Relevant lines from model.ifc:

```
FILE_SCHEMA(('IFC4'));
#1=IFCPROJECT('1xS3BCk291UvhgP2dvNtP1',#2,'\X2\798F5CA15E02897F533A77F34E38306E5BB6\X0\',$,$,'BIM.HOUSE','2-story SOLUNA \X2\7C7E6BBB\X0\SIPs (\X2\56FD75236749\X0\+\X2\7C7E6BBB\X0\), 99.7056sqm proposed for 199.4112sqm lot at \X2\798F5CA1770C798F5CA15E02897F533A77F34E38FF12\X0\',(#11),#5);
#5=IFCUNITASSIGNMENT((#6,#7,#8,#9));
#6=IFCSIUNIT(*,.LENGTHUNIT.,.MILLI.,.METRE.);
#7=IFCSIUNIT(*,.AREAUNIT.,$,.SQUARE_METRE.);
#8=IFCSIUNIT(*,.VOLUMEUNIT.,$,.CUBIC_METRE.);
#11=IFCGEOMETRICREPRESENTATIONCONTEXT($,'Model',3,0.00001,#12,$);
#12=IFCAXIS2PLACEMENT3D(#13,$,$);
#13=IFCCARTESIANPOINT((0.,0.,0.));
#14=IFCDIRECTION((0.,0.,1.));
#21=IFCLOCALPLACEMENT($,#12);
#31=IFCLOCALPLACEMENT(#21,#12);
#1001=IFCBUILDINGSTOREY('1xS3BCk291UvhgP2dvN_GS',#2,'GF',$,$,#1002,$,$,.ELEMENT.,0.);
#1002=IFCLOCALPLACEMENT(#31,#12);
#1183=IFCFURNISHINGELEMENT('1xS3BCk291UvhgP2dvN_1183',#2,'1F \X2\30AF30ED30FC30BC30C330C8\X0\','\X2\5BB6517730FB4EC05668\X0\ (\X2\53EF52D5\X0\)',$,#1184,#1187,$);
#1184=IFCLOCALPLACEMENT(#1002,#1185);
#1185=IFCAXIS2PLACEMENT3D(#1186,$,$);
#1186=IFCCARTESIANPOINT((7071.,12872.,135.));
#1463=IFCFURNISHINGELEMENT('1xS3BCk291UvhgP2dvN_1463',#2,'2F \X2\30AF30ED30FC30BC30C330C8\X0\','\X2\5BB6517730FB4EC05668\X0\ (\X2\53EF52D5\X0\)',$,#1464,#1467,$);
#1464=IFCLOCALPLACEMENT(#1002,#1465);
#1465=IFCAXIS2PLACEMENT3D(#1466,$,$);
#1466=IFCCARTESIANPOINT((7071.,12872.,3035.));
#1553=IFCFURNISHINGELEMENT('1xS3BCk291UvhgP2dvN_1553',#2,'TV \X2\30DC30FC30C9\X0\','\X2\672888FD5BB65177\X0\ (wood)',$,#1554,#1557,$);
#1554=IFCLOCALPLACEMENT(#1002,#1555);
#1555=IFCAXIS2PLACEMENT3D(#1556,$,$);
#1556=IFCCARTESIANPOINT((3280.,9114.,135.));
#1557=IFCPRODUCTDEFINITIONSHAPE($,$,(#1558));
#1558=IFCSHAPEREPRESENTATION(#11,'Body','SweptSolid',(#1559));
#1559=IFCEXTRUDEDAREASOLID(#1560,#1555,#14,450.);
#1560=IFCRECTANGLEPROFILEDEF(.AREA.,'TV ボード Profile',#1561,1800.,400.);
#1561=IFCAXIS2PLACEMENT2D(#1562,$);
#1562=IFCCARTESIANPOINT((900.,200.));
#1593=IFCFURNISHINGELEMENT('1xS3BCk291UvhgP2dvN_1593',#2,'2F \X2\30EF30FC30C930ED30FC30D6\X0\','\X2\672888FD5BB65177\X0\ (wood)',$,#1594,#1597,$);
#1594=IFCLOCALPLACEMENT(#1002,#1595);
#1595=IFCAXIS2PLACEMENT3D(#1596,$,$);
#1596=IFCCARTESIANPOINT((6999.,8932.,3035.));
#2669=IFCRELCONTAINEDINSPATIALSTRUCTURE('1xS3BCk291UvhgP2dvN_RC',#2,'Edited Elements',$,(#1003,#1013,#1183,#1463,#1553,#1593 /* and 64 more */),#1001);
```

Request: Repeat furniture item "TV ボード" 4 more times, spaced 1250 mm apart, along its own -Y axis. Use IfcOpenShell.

```python
import ifcopenshell
import ifcopenshell.api.geometry
import ifcopenshell.api.root
import ifcopenshell.util.element
import ifcopenshell.util.placement
import ifcopenshell.util.unit

model = ifcopenshell.open("model.ifc")
unit_scale = ifcopenshell.util.unit.calculate_unit_scale(model)


def reuse_history(source, copy):
    """copy_class also copies each property set's owner history, people and application; keep the originals."""
    for rel in copy.IsDefinedBy:
        if rel.is_a("IfcRelDefinesByProperties") and (history := rel.RelatingPropertyDefinition.OwnerHistory):
            rel.RelatingPropertyDefinition.OwnerHistory = source.OwnerHistory
            ifcopenshell.util.element.remove_deep2(model, history)


source = model.by_guid("1xS3BCk291UvhgP2dvN_1553")
base = ifcopenshell.util.placement.get_local_placement(source.ObjectPlacement)
step = -base[:3, 1] * 1.25 / unit_scale

for i in range(1, 5):
    copy = ifcopenshell.api.root.copy_class(model, product=source)
    copy.Representation = ifcopenshell.util.element.copy_deep(
        model, source.Representation, exclude=["IfcGeometricRepresentationContext", "IfcRepresentationMap"]
    )
    reuse_history(source, copy)
    matrix = base.copy()
    matrix[:3, 3] += i * step
    print("added at", matrix[:3, 3].round(3) + 0.0)
    ifcopenshell.api.geometry.edit_object_placement(model, product=copy, matrix=matrix, is_si=False)

model.write("model-out.ifc")
```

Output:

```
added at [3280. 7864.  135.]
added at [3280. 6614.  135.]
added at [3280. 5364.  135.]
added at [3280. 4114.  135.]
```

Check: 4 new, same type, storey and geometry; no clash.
